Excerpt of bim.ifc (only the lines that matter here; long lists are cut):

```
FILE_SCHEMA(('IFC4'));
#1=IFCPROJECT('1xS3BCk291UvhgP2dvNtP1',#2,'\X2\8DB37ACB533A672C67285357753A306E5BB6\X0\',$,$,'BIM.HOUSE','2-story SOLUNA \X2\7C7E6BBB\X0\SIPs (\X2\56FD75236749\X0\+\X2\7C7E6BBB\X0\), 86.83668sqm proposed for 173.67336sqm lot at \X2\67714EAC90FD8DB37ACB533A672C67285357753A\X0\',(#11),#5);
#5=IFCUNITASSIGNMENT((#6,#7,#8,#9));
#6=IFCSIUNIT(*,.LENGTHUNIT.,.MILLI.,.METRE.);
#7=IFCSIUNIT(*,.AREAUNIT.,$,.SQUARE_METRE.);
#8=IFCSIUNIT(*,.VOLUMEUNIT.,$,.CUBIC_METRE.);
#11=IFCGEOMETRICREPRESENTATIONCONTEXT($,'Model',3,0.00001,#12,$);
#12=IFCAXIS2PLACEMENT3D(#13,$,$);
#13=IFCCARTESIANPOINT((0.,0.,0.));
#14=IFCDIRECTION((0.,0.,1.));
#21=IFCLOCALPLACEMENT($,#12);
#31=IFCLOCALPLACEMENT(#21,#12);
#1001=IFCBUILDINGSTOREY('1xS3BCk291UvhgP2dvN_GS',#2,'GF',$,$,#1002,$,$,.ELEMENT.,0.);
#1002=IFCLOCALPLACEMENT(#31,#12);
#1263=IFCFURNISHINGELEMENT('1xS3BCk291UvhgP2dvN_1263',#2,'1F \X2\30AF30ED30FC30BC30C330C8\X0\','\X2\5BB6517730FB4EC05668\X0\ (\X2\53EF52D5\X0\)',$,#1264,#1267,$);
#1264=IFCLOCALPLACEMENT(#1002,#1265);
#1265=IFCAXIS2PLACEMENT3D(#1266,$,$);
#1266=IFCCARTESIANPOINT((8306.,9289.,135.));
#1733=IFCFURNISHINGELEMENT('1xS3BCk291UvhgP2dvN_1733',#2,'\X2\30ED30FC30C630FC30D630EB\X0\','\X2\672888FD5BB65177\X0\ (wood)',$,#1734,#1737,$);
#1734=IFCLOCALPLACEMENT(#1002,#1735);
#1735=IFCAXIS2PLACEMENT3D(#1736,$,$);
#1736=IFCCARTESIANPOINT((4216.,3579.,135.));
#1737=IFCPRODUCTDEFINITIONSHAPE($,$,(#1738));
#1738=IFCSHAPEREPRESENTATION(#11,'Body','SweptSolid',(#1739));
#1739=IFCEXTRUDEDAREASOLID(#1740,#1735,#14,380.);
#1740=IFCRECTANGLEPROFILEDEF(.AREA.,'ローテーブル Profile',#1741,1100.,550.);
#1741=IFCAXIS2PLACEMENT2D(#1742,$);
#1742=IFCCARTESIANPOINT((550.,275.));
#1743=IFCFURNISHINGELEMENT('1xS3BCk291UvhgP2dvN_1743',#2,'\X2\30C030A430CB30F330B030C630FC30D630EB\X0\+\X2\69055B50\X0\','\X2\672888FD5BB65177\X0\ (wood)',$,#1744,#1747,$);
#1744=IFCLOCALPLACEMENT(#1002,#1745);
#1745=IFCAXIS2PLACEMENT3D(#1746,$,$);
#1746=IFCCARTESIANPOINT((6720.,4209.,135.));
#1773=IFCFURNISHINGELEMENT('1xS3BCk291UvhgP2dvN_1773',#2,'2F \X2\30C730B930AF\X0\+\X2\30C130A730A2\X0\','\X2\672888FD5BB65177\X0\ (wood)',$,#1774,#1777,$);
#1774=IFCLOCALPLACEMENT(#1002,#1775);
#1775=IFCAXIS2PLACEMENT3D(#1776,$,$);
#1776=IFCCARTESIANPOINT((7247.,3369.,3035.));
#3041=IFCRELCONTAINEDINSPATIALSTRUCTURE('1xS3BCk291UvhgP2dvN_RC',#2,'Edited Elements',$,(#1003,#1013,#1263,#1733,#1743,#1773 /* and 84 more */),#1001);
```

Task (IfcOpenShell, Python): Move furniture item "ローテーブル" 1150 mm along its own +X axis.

```python
import ifcopenshell
import ifcopenshell.api.geometry
import ifcopenshell.util.placement
import ifcopenshell.util.unit

model = ifcopenshell.open("bim.ifc")
unit_scale = ifcopenshell.util.unit.calculate_unit_scale(model)

item = model.by_guid("1xS3BCk291UvhgP2dvN_1733")
matrix = ifcopenshell.util.placement.get_local_placement(item.ObjectPlacement)
matrix[:3, 3] += matrix[:3, 0] * 1.15 / unit_scale
ifcopenshell.api.geometry.edit_object_placement(model, product=item, matrix=matrix, is_si=False)

print(ifcopenshell.util.placement.get_local_placement(item.ObjectPlacement).round(3) + 0.0)

model.write("bim_edited.ifc")
```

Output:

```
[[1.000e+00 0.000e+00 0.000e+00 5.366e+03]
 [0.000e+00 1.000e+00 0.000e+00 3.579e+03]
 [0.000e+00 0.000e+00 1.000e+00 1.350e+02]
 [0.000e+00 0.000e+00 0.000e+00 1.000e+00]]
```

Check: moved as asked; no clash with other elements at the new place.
